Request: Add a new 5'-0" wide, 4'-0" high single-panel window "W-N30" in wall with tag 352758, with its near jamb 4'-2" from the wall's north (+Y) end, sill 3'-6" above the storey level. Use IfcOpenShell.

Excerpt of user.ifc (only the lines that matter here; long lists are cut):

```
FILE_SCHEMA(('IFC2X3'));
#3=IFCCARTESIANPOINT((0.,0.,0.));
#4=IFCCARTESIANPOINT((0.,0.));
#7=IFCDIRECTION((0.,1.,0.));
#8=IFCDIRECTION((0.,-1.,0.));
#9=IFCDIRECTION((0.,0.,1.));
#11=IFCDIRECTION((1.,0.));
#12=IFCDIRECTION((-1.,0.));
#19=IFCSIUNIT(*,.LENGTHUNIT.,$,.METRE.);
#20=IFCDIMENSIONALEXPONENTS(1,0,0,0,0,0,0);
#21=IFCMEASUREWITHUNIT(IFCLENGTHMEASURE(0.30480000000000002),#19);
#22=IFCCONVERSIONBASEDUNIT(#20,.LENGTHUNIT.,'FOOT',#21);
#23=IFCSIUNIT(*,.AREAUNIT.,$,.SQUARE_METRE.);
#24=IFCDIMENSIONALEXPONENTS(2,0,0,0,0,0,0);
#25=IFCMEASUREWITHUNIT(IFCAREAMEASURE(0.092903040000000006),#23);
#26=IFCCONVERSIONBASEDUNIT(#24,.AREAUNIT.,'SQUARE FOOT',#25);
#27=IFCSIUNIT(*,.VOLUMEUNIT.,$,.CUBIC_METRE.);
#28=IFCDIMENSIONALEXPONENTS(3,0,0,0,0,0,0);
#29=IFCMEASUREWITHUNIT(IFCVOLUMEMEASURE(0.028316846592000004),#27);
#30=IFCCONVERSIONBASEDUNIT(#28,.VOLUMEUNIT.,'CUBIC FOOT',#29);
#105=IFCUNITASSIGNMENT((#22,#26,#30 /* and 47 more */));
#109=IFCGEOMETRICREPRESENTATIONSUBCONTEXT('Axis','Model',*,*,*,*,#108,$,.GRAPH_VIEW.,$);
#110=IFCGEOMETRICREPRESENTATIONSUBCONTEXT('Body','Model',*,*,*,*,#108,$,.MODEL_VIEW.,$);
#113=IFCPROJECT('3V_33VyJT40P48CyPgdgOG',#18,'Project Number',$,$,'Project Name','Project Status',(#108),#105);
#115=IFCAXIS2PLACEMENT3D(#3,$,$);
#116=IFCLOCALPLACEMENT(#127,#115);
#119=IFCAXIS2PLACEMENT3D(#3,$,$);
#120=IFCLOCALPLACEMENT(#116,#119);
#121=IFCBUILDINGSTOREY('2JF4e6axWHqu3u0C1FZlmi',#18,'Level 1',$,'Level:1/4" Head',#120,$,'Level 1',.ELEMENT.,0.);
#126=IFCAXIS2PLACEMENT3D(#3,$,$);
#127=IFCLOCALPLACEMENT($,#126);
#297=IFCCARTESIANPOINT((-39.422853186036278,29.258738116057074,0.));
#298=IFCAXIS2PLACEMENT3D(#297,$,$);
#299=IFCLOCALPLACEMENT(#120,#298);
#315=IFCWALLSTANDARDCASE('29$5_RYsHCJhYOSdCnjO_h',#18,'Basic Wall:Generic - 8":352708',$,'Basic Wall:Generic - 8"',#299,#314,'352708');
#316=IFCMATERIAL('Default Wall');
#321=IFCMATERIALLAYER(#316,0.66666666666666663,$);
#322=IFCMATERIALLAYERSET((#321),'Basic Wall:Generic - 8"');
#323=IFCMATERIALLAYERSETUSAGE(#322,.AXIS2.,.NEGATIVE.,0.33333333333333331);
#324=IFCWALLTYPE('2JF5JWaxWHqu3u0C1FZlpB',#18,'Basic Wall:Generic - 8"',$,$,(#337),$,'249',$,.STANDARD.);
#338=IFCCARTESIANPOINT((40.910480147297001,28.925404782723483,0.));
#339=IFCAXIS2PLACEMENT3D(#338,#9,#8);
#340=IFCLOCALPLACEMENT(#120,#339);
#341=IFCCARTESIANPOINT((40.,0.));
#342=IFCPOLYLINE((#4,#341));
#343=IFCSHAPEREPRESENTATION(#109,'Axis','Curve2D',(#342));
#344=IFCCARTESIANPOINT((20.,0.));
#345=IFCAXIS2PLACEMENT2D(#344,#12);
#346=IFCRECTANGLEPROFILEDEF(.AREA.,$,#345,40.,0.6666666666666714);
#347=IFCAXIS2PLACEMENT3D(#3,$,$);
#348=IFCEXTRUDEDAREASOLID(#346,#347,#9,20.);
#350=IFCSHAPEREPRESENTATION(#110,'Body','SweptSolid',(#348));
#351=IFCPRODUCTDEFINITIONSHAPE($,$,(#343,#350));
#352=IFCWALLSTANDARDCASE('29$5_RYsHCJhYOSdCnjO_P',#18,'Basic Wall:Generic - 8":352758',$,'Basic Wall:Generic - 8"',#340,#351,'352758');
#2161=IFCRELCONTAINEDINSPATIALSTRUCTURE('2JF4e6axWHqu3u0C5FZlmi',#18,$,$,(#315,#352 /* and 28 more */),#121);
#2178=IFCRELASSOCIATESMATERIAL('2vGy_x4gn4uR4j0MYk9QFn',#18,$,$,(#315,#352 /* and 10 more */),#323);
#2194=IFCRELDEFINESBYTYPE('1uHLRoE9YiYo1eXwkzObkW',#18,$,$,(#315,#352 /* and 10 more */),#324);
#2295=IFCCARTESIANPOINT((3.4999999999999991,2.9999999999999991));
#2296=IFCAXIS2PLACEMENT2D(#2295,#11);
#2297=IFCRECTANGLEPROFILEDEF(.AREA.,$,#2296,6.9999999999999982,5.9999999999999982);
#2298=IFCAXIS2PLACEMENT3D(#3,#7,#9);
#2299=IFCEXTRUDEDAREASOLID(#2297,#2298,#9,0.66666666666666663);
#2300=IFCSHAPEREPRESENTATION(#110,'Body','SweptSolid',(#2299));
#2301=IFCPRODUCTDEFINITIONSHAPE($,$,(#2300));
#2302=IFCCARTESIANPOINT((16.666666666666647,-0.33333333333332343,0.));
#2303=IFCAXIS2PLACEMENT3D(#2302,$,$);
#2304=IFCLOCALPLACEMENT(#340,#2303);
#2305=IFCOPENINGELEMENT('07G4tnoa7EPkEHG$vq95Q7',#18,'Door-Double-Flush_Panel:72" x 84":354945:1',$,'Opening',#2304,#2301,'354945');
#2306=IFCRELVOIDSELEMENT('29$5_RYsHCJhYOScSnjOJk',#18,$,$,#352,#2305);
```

```python
import numpy as np
import ifcopenshell
import ifcopenshell.api.feature
import ifcopenshell.api.geometry
import ifcopenshell.api.root
import ifcopenshell.api.spatial
import ifcopenshell.api.type
import ifcopenshell.geom
import ifcopenshell.util.element
import ifcopenshell.util.placement
import ifcopenshell.util.representation
import ifcopenshell.util.shape
import ifcopenshell.util.unit

model = ifcopenshell.open("user.ifc")
unit_scale = ifcopenshell.util.unit.calculate_unit_scale(model)
settings = ifcopenshell.geom.settings()


def volume(element):
    """Net volume in cubic metres, openings subtracted."""
    shape = ifcopenshell.geom.create_shape(settings, element)
    return ifcopenshell.util.shape.get_volume(shape.geometry)


wall = model.by_guid("29$5_RYsHCJhYOSdCnjO_P")
storey = ifcopenshell.util.element.get_container(wall, ifc_class="IfcBuildingStorey")
context = ifcopenshell.util.representation.get_context(model, "Model", "Body", "MODEL_VIEW")
before = volume(wall)

width, height, from_end, sill = 1.524, 1.2192, 1.27, 1.0668  # metres

# The wall runs along its own X axis, and the end named is its -X end.
wall_shape = ifcopenshell.geom.create_shape(settings, wall)
x, y, z = ifcopenshell.util.shape.get_vertices(wall_shape.geometry).T
start = x.min() + from_end
face, thickness = float(y.min()), float(y.max() - y.min())
wall_matrix = ifcopenshell.util.placement.get_local_placement(wall.ObjectPlacement)
level = ifcopenshell.util.placement.get_local_placement(storey.ObjectPlacement)[2, 3]


def in_wall(x, y):
    """Placement at x, y metres in the wall's axes, at sill height."""
    matrix = wall_matrix.copy()
    matrix[:, 3] = wall_matrix @ np.array([x / unit_scale, y / unit_scale, 0.0, 1.0])
    matrix[2, 3] = level + sill / unit_scale
    return matrix


# Opening: a box that overshoots both wall faces by 50 mm.
opening = ifcopenshell.api.root.create_entity(model, ifc_class="IfcOpeningElement")
box = ifcopenshell.api.geometry.add_wall_representation(
    model, context=context, length=width, height=height, thickness=thickness + 0.1
)
ifcopenshell.api.geometry.assign_representation(model, product=opening, representation=box)
ifcopenshell.api.geometry.edit_object_placement(model, product=opening, matrix=in_wall(start, face - 0.05), is_si=False)
ifcopenshell.api.feature.add_feature(model, feature=opening, element=wall)

window = ifcopenshell.api.root.create_entity(model, ifc_class="IfcWindow", name="W-N30")
window.OverallWidth, window.OverallHeight = width / unit_scale, height / unit_scale
body = ifcopenshell.api.geometry.add_window_representation(
    model,
    context=context,
    overall_width=window.OverallWidth,
    overall_height=window.OverallHeight,
    partition_type="SINGLE_PANEL",
)
ifcopenshell.api.geometry.assign_representation(model, product=window, representation=body)
ifcopenshell.api.spatial.assign_container(model, products=[window], relating_structure=storey)
fills = ifcopenshell.api.feature.add_filling(model, opening=opening, element=window)
fills.OwnerHistory = window.OwnerHistory  # required in IFC2X3

# IFC2X3 keeps the operation on the window style.
style = ifcopenshell.api.root.create_entity(model, ifc_class="IfcWindowStyle", name="W-N30")
style.OperationType, style.ConstructionType = "SINGLE_PANEL", "NOTDEFINED"
style.ParameterTakesPrecedence = style.Sizeable = False
ifcopenshell.api.type.assign_type(model, related_objects=[window], relating_type=style)

# Centre the window in the wall's thickness.
ifcopenshell.api.geometry.edit_object_placement(model, product=window, matrix=in_wall(start, face), is_si=False)
window_shape = ifcopenshell.geom.create_shape(settings, window)
depth = ifcopenshell.util.shape.get_vertices(window_shape.geometry)[:, 1]
offset = face + thickness / 2 - (depth.min() + depth.max()) / 2
ifcopenshell.api.geometry.edit_object_placement(model, product=window, matrix=in_wall(start, offset), is_si=False)

after = volume(wall)

print(f"wall volume {before:.3f} -> {after:.3f} m3")

model.write("user_edited.ifc")
```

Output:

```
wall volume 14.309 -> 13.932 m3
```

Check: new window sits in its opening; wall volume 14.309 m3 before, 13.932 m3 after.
